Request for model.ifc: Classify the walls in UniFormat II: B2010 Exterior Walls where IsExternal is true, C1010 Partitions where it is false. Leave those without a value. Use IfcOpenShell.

First a look at what the model holds.

```python
import ifcopenshell
import ifcopenshell.util.element

model = ifcopenshell.open("model.ifc")
print(model.schema)
print("classifications:", [c.Name for c in model.by_type("IfcClassification")])
values = [ifcopenshell.util.element.get_pset(e, "Pset_WallCommon", "IsExternal") for e in model.by_type("IfcWall")]
for value in (True, False, None):
    print("IsExternal", value, values.count(value))
```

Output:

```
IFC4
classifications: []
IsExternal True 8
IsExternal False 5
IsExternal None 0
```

```python
import ifcopenshell
import ifcopenshell.api.classification
import ifcopenshell.util.element

model = ifcopenshell.open("model.ifc")

system = ifcopenshell.api.classification.add_classification(model, classification="UniFormat II")

walls = model.by_type("IfcWall")
external = {e: ifcopenshell.util.element.get_pset(e, "Pset_WallCommon", "IsExternal") for e in walls}
for flag, code, name in ((True, "B2010", "Exterior Walls"), (False, "C1010", "Partitions")):
    products = [e for e in walls if external[e] is flag]
    ifcopenshell.api.classification.add_reference(
        model, products=products, classification=system, identification=code, name=name
    )
    print(code, len(products))

model.write("model-out.ifc")
```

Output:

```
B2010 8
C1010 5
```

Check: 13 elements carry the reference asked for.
